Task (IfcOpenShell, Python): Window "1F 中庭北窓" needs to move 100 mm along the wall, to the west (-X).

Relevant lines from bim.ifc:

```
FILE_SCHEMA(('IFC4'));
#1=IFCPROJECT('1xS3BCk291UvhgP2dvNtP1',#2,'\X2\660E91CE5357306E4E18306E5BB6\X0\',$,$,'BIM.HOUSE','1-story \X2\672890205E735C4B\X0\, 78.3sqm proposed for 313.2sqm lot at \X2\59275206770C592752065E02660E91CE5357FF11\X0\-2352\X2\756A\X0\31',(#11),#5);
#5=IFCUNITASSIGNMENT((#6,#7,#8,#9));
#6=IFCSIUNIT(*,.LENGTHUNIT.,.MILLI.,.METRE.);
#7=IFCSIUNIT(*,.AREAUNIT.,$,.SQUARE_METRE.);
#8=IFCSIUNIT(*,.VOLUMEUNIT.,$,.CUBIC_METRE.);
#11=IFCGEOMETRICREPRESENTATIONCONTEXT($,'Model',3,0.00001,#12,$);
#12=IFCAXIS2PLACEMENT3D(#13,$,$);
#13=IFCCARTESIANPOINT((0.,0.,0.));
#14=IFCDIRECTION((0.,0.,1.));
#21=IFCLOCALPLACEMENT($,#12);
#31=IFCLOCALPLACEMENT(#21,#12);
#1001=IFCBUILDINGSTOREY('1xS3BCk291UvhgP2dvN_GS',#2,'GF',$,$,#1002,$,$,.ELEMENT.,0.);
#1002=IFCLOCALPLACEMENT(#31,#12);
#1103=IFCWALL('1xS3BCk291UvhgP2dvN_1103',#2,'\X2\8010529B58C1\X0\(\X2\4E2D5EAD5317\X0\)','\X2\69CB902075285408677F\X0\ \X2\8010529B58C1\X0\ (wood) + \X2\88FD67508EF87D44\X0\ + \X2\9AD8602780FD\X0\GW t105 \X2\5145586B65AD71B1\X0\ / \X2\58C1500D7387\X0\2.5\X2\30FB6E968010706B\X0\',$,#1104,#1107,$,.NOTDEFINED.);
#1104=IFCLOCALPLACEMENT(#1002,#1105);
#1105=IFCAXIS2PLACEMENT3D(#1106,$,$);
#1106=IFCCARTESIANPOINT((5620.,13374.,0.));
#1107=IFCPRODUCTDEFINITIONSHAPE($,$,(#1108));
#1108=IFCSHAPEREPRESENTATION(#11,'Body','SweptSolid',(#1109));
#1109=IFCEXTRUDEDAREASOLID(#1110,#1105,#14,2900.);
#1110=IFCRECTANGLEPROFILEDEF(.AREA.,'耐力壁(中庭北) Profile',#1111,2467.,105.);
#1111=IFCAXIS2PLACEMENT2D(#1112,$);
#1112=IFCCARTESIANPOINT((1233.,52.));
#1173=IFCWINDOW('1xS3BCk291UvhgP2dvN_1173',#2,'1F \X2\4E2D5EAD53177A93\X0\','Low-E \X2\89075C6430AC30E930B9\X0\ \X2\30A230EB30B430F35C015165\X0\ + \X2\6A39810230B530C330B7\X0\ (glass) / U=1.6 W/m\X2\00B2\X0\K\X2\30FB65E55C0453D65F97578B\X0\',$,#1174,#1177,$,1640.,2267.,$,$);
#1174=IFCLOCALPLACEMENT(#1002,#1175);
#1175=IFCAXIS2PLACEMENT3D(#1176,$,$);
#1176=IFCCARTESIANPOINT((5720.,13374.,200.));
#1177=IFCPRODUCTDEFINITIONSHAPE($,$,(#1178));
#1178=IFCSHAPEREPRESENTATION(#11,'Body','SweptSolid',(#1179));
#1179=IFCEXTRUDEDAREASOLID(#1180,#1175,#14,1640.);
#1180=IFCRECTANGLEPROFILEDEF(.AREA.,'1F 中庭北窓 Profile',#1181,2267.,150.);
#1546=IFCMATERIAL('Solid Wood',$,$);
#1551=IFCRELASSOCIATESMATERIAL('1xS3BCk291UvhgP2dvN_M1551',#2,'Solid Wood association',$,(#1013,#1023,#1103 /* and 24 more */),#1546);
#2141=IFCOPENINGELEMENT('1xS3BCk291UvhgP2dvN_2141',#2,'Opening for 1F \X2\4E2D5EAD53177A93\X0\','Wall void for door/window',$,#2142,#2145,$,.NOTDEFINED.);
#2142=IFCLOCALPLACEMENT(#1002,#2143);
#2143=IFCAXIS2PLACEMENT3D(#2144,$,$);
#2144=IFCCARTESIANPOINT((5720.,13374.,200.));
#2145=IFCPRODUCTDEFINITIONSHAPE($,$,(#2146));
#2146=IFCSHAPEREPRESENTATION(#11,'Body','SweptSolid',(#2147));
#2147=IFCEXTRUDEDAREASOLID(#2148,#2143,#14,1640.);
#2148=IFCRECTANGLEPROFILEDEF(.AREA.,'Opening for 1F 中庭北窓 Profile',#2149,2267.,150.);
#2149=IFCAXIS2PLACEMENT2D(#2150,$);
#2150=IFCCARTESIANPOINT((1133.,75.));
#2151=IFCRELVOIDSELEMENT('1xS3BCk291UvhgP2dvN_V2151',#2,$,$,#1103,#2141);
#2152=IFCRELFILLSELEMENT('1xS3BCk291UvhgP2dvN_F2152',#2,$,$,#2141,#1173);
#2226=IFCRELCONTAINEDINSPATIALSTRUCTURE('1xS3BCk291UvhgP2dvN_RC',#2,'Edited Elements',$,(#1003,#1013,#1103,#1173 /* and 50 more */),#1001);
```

```python
import ifcopenshell
import ifcopenshell.api.geometry
import ifcopenshell.util.placement

model = ifcopenshell.open("bim.ifc")

window = model.by_guid("1xS3BCk291UvhgP2dvN_1173")
opening = window.FillsVoids[0].RelatingOpeningElement
wall = opening.VoidsElements[0].RelatingBuildingElement

wall_matrix = ifcopenshell.util.placement.get_local_placement(wall.ObjectPlacement)
shift = wall_matrix[:3, 0] * -100.0
before = ifcopenshell.util.placement.get_local_placement(window.ObjectPlacement)[:3, 3].copy()

# The window is not placed relative to its opening, so move both.
for product in (opening, window):
    matrix = ifcopenshell.util.placement.get_local_placement(product.ObjectPlacement)
    matrix[:3, 3] += shift
    ifcopenshell.api.geometry.edit_object_placement(model, product=product, matrix=matrix, is_si=False)

after = ifcopenshell.util.placement.get_local_placement(window.ObjectPlacement)[:3, 3]
print("window moved by", (after - before).round(3) + 0.0)

model.write("bim_updated.ifc")
```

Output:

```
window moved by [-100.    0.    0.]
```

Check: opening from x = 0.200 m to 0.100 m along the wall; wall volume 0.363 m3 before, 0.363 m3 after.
